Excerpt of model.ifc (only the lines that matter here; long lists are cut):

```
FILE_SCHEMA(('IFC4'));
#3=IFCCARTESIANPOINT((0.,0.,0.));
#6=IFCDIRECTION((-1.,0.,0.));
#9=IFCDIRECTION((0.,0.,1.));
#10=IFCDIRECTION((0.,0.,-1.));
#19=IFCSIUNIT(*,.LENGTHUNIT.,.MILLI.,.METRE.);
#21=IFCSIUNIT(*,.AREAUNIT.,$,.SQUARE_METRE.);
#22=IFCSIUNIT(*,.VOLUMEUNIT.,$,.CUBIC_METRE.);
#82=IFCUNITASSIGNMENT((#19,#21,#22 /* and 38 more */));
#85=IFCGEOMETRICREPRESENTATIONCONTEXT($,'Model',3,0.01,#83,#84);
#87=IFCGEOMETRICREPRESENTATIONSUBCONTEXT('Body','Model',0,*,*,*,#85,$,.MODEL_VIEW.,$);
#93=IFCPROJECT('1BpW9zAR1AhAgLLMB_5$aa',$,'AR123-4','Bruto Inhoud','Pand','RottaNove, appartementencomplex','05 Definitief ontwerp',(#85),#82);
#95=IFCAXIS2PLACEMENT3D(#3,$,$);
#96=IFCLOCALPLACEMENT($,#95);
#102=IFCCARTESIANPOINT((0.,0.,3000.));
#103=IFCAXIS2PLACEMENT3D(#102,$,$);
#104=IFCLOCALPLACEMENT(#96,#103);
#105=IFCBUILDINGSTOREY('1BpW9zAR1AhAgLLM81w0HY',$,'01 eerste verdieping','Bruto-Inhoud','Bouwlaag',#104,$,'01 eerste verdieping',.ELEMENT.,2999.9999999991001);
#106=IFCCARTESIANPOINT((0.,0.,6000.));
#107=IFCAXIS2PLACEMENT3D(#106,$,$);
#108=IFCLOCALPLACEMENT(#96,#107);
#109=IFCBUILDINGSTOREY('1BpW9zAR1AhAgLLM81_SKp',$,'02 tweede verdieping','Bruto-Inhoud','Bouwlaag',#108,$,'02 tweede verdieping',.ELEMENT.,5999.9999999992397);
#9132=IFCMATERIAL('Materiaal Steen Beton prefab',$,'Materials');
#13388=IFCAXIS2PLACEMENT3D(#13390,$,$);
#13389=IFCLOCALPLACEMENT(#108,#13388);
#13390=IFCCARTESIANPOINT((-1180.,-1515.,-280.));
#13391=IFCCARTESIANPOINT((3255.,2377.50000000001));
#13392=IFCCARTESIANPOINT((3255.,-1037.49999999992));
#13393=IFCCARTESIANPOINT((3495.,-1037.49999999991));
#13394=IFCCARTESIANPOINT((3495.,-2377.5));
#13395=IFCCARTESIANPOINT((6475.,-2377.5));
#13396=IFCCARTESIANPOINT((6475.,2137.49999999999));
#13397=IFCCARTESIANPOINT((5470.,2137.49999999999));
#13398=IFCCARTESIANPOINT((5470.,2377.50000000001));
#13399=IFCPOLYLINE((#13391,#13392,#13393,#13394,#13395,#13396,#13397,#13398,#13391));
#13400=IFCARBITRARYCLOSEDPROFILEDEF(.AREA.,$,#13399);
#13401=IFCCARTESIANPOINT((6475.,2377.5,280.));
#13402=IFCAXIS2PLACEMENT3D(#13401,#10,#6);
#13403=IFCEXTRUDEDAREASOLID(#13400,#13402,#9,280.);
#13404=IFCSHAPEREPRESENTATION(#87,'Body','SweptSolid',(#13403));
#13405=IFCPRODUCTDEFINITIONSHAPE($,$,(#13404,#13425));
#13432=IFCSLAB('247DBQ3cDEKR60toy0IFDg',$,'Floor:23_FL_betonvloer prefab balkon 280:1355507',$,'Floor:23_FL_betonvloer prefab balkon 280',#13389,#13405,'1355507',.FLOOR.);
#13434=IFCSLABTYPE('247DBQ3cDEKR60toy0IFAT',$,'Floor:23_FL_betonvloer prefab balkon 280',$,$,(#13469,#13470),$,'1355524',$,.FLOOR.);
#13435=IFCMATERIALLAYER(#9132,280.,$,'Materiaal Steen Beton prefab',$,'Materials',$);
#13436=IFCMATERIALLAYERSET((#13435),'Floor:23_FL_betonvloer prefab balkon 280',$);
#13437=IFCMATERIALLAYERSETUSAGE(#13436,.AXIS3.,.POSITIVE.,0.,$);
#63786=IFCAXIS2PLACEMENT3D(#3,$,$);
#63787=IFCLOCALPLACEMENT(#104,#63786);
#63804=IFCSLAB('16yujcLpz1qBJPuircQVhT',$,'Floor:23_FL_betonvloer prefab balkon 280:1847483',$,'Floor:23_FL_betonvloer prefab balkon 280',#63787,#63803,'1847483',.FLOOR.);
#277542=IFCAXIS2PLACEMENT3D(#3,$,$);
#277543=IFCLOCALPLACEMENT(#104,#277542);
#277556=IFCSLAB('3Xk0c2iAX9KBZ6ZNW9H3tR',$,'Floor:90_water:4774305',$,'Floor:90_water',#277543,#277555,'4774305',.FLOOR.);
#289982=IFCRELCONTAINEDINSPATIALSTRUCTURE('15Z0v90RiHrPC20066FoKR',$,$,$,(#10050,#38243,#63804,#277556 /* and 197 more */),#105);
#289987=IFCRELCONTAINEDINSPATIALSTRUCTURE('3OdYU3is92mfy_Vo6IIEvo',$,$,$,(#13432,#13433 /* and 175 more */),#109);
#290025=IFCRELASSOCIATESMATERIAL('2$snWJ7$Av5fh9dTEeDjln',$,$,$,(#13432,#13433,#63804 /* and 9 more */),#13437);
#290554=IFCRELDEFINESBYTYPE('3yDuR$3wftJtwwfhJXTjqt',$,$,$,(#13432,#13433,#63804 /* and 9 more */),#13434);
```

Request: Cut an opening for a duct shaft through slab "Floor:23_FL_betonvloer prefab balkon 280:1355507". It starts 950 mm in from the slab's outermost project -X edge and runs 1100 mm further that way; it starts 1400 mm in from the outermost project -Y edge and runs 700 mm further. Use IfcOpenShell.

```python
import numpy as np
import ifcopenshell
import ifcopenshell.api.feature
import ifcopenshell.api.geometry
import ifcopenshell.api.root
import ifcopenshell.geom
import ifcopenshell.util.placement
import ifcopenshell.util.representation
import ifcopenshell.util.shape
import ifcopenshell.util.unit

model = ifcopenshell.open("model.ifc")
unit_scale = ifcopenshell.util.unit.calculate_unit_scale(model)
settings = ifcopenshell.geom.settings()


def volume(element):
    """Net volume in cubic metres, openings subtracted."""
    shape = ifcopenshell.geom.create_shape(settings, element)
    return ifcopenshell.util.shape.get_volume(shape.geometry)


slab = model.by_id(13432)
before = volume(slab)

# Extent in the slab's own axes, in metres. The edges named are its -X and -Y sides.
slab_shape = ifcopenshell.geom.create_shape(settings, slab)
vertices = ifcopenshell.util.shape.get_vertices(slab_shape.geometry)
x_min, y_min, bottom = vertices.min(axis=0)
top = vertices[:, 2].max()

opening = ifcopenshell.api.root.create_entity(model, ifc_class="IfcOpeningElement", name="Duct shaft opening", predefined_type="OPENING")
context = ifcopenshell.util.representation.get_context(model, "Model", "Body", "MODEL_VIEW")
width, depth = 1.1, 0.7
outline = [(0.0, 0.0), (width, 0.0), (width, depth), (0.0, depth), (0.0, 0.0)]
# Overshoot both faces by 50 mm so the cut is clean.
shape = ifcopenshell.api.geometry.add_slab_representation(
    model, context=context, depth=top - bottom + 0.1, polyline=outline
)
ifcopenshell.api.geometry.assign_representation(model, product=opening, representation=shape)

matrix = ifcopenshell.util.placement.get_local_placement(slab.ObjectPlacement)
matrix[:, 3] = matrix @ np.append(np.array([x_min + 0.95, y_min + 1.4, bottom - 0.05]) / unit_scale, 1.0)
ifcopenshell.api.geometry.edit_object_placement(model, product=opening, matrix=matrix, is_si=False)
ifcopenshell.api.feature.add_feature(model, feature=opening, element=slab)

after = volume(slab)

print(f"slab volume {before:.3f} -> {after:.3f} m3")

model.write("model_updated.ifc")
```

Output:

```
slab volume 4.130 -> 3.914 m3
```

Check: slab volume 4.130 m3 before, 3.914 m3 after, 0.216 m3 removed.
